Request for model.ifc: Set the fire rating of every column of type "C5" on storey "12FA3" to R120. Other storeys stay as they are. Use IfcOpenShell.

First a look at what the model holds.

```python
import ifcopenshell
import ifcopenshell.util.element

model = ifcopenshell.open("model.ifc")
print(model.schema)
storey = next(s for s in model.by_type("IfcBuildingStorey") if s.Name == "12FA3")
columns = [e for e in ifcopenshell.util.element.get_decomposition(storey) if e.is_a("IfcColumn")]
seen = {}
for e in columns:
    element_type = ifcopenshell.util.element.get_type(e)
    key = (element_type.Name if element_type != e and element_type else None, ifcopenshell.util.element.get_pset(e, "Pset_ColumnCommon", "FireRating"))
    seen[key] = seen.get(key, 0) + 1
for (name, value), count in sorted(seen.items(), key=str):
    print(count, "x", name, "|", value)
```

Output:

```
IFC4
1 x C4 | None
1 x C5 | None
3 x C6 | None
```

```python
import ifcopenshell
import ifcopenshell.api.pset
import ifcopenshell.util.element

model = ifcopenshell.open("model.ifc")

storey = next(s for s in model.by_type("IfcBuildingStorey") if s.Name == "12FA3")
columns = [e for e in ifcopenshell.util.element.get_decomposition(storey) if e.is_a("IfcColumn")]

count = 0
for e in columns:
    element_type = ifcopenshell.util.element.get_type(e)
    if element_type in (None, e) or element_type.Name != "C5":
        continue
    # add_pset returns the element's existing set when there is one.
    pset = ifcopenshell.api.pset.add_pset(model, product=e, name="Pset_ColumnCommon")
    ifcopenshell.api.pset.edit_pset(model, pset=pset, properties={"FireRating": "R120"})
    count += 1

print(count, "columns updated")

model.write("model_rev.ifc")
```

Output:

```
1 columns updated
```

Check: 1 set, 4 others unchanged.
